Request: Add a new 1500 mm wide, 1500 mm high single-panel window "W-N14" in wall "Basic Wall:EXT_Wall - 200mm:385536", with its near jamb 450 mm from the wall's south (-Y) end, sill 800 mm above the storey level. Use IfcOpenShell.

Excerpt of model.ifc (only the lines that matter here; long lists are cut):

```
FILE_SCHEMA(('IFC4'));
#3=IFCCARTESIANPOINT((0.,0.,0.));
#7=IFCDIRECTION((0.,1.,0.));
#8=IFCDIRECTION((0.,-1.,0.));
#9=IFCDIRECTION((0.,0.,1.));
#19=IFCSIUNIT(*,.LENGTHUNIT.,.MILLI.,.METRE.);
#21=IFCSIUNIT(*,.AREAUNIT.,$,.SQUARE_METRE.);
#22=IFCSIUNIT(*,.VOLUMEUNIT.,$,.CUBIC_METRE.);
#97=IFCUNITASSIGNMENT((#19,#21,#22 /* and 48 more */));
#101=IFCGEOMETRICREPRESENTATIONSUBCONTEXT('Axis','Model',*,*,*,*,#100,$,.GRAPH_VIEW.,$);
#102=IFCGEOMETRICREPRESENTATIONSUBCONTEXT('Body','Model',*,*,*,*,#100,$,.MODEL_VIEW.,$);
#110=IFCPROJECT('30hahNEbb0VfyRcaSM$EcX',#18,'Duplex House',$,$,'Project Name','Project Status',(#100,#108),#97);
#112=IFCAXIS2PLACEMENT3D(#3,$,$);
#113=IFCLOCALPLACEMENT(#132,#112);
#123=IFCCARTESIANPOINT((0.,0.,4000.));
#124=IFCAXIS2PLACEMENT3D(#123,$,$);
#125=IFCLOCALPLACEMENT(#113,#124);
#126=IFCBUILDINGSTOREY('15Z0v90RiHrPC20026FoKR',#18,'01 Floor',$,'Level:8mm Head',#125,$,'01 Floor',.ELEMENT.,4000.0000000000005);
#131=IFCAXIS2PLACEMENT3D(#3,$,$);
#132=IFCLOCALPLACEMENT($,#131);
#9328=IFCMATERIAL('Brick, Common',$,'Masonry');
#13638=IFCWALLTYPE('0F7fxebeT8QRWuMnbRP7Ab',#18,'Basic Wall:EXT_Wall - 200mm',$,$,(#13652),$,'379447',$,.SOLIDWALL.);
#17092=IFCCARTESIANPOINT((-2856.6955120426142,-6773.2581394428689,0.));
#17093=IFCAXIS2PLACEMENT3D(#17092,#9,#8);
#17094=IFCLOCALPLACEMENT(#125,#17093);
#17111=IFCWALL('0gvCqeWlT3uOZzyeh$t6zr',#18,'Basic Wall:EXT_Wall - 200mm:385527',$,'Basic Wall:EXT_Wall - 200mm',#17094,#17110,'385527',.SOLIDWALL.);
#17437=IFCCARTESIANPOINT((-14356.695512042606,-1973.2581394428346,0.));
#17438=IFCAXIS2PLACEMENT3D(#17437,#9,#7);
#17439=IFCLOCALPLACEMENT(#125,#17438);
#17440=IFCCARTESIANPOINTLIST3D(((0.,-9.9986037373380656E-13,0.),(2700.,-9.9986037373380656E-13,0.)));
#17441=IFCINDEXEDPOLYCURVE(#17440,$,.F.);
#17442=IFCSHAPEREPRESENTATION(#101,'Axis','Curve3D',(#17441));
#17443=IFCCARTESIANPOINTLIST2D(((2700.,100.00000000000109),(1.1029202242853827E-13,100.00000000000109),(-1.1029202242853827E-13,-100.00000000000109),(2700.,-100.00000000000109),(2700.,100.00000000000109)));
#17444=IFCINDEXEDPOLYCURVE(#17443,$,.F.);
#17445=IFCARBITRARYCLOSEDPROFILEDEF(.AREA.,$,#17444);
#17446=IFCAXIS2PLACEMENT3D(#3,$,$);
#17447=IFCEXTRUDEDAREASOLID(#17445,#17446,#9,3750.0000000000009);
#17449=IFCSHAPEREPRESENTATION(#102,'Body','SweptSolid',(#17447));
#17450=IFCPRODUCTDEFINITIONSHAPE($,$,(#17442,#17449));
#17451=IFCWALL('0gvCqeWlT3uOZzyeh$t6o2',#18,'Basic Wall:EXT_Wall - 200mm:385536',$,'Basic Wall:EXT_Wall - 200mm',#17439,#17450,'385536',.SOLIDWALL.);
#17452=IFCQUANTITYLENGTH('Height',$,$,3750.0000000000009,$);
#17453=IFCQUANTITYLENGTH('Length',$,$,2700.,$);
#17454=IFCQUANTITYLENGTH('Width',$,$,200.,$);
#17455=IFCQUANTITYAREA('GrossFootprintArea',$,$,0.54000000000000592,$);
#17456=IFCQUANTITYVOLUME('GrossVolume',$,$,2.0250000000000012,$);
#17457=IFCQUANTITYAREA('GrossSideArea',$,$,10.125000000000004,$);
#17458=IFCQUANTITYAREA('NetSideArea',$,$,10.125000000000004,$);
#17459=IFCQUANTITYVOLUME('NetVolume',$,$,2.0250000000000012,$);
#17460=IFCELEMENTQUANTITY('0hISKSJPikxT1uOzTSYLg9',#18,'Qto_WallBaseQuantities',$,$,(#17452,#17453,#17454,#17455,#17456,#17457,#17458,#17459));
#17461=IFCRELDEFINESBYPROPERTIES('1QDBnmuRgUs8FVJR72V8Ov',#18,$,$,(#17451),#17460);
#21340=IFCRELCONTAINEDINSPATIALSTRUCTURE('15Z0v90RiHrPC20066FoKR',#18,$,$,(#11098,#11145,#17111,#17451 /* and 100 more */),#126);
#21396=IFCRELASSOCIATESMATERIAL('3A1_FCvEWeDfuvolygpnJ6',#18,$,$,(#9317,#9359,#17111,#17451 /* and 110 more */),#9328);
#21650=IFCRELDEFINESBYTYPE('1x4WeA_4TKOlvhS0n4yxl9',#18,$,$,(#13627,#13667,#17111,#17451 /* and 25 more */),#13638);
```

```python
import numpy as np
import ifcopenshell
import ifcopenshell.api.feature
import ifcopenshell.api.geometry
import ifcopenshell.api.pset
import ifcopenshell.api.root
import ifcopenshell.api.spatial
import ifcopenshell.geom
import ifcopenshell.util.element
import ifcopenshell.util.placement
import ifcopenshell.util.representation
import ifcopenshell.util.shape
import ifcopenshell.util.unit

model = ifcopenshell.open("model.ifc")
unit_scale = ifcopenshell.util.unit.calculate_unit_scale(model)
area_scale = ifcopenshell.util.unit.calculate_unit_scale(model, "AREAUNIT")
volume_scale = ifcopenshell.util.unit.calculate_unit_scale(model, "VOLUMEUNIT")
settings = ifcopenshell.geom.settings()


def volume(element):
    """Net volume in cubic metres, openings subtracted."""
    shape = ifcopenshell.geom.create_shape(settings, element)
    return ifcopenshell.util.shape.get_volume(shape.geometry)


wall = model.by_guid("0gvCqeWlT3uOZzyeh$t6o2")
storey = ifcopenshell.util.element.get_container(wall, ifc_class="IfcBuildingStorey")
context = ifcopenshell.util.representation.get_context(model, "Model", "Body", "MODEL_VIEW")
before = volume(wall)

width, height, from_end, sill = 1.5, 1.5, 0.45, 0.8  # metres

# The wall runs along its own X axis, and the end named is its -X end.
wall_shape = ifcopenshell.geom.create_shape(settings, wall)
x, y, z = ifcopenshell.util.shape.get_vertices(wall_shape.geometry).T
start = x.min() + from_end
face, thickness = float(y.min()), float(y.max() - y.min())
wall_matrix = ifcopenshell.util.placement.get_local_placement(wall.ObjectPlacement)
level = ifcopenshell.util.placement.get_local_placement(storey.ObjectPlacement)[2, 3]


def in_wall(x, y):
    """Placement at x, y metres in the wall's axes, at sill height."""
    matrix = wall_matrix.copy()
    matrix[:, 3] = wall_matrix @ np.array([x / unit_scale, y / unit_scale, 0.0, 1.0])
    matrix[2, 3] = level + sill / unit_scale
    return matrix


# Opening: a box that overshoots both wall faces by 50 mm.
opening = ifcopenshell.api.root.create_entity(model, ifc_class="IfcOpeningElement", predefined_type="OPENING")
box = ifcopenshell.api.geometry.add_wall_representation(
    model, context=context, length=width, height=height, thickness=thickness + 0.1
)
ifcopenshell.api.geometry.assign_representation(model, product=opening, representation=box)
ifcopenshell.api.geometry.edit_object_placement(model, product=opening, matrix=in_wall(start, face - 0.05), is_si=False)
ifcopenshell.api.feature.add_feature(model, feature=opening, element=wall)

window = ifcopenshell.api.root.create_entity(model, ifc_class="IfcWindow", name="W-N14", predefined_type="WINDOW")
window.OverallWidth, window.OverallHeight = width / unit_scale, height / unit_scale
window.PartitioningType = "SINGLE_PANEL"
body = ifcopenshell.api.geometry.add_window_representation(
    model,
    context=context,
    overall_width=window.OverallWidth,
    overall_height=window.OverallHeight,
    partition_type="SINGLE_PANEL",
)
ifcopenshell.api.geometry.assign_representation(model, product=window, representation=body)
ifcopenshell.api.spatial.assign_container(model, products=[window], relating_structure=storey)
ifcopenshell.api.feature.add_filling(model, opening=opening, element=window)

# Centre the window in the wall's thickness.
ifcopenshell.api.geometry.edit_object_placement(model, product=window, matrix=in_wall(start, face), is_si=False)
window_shape = ifcopenshell.geom.create_shape(settings, window)
depth = ifcopenshell.util.shape.get_vertices(window_shape.geometry)[:, 1]
offset = face + thickness / 2 - (depth.min() + depth.max()) / 2
ifcopenshell.api.geometry.edit_object_placement(model, product=window, matrix=in_wall(start, offset), is_si=False)

after = volume(wall)

# Update the wall's stored quantities.
qto = model.by_id(ifcopenshell.util.element.get_pset(wall, "Qto_WallBaseQuantities", should_inherit=False)["id"])
ifcopenshell.api.pset.edit_qto(model, qto=qto, properties={
    "NetSideArea": after / thickness / area_scale,
    "NetVolume": after / volume_scale,
})

print(f"wall volume {before:.3f} -> {after:.3f} m3")

model.write("model_updated.ifc")
```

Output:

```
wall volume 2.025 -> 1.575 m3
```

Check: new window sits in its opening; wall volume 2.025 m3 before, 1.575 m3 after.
